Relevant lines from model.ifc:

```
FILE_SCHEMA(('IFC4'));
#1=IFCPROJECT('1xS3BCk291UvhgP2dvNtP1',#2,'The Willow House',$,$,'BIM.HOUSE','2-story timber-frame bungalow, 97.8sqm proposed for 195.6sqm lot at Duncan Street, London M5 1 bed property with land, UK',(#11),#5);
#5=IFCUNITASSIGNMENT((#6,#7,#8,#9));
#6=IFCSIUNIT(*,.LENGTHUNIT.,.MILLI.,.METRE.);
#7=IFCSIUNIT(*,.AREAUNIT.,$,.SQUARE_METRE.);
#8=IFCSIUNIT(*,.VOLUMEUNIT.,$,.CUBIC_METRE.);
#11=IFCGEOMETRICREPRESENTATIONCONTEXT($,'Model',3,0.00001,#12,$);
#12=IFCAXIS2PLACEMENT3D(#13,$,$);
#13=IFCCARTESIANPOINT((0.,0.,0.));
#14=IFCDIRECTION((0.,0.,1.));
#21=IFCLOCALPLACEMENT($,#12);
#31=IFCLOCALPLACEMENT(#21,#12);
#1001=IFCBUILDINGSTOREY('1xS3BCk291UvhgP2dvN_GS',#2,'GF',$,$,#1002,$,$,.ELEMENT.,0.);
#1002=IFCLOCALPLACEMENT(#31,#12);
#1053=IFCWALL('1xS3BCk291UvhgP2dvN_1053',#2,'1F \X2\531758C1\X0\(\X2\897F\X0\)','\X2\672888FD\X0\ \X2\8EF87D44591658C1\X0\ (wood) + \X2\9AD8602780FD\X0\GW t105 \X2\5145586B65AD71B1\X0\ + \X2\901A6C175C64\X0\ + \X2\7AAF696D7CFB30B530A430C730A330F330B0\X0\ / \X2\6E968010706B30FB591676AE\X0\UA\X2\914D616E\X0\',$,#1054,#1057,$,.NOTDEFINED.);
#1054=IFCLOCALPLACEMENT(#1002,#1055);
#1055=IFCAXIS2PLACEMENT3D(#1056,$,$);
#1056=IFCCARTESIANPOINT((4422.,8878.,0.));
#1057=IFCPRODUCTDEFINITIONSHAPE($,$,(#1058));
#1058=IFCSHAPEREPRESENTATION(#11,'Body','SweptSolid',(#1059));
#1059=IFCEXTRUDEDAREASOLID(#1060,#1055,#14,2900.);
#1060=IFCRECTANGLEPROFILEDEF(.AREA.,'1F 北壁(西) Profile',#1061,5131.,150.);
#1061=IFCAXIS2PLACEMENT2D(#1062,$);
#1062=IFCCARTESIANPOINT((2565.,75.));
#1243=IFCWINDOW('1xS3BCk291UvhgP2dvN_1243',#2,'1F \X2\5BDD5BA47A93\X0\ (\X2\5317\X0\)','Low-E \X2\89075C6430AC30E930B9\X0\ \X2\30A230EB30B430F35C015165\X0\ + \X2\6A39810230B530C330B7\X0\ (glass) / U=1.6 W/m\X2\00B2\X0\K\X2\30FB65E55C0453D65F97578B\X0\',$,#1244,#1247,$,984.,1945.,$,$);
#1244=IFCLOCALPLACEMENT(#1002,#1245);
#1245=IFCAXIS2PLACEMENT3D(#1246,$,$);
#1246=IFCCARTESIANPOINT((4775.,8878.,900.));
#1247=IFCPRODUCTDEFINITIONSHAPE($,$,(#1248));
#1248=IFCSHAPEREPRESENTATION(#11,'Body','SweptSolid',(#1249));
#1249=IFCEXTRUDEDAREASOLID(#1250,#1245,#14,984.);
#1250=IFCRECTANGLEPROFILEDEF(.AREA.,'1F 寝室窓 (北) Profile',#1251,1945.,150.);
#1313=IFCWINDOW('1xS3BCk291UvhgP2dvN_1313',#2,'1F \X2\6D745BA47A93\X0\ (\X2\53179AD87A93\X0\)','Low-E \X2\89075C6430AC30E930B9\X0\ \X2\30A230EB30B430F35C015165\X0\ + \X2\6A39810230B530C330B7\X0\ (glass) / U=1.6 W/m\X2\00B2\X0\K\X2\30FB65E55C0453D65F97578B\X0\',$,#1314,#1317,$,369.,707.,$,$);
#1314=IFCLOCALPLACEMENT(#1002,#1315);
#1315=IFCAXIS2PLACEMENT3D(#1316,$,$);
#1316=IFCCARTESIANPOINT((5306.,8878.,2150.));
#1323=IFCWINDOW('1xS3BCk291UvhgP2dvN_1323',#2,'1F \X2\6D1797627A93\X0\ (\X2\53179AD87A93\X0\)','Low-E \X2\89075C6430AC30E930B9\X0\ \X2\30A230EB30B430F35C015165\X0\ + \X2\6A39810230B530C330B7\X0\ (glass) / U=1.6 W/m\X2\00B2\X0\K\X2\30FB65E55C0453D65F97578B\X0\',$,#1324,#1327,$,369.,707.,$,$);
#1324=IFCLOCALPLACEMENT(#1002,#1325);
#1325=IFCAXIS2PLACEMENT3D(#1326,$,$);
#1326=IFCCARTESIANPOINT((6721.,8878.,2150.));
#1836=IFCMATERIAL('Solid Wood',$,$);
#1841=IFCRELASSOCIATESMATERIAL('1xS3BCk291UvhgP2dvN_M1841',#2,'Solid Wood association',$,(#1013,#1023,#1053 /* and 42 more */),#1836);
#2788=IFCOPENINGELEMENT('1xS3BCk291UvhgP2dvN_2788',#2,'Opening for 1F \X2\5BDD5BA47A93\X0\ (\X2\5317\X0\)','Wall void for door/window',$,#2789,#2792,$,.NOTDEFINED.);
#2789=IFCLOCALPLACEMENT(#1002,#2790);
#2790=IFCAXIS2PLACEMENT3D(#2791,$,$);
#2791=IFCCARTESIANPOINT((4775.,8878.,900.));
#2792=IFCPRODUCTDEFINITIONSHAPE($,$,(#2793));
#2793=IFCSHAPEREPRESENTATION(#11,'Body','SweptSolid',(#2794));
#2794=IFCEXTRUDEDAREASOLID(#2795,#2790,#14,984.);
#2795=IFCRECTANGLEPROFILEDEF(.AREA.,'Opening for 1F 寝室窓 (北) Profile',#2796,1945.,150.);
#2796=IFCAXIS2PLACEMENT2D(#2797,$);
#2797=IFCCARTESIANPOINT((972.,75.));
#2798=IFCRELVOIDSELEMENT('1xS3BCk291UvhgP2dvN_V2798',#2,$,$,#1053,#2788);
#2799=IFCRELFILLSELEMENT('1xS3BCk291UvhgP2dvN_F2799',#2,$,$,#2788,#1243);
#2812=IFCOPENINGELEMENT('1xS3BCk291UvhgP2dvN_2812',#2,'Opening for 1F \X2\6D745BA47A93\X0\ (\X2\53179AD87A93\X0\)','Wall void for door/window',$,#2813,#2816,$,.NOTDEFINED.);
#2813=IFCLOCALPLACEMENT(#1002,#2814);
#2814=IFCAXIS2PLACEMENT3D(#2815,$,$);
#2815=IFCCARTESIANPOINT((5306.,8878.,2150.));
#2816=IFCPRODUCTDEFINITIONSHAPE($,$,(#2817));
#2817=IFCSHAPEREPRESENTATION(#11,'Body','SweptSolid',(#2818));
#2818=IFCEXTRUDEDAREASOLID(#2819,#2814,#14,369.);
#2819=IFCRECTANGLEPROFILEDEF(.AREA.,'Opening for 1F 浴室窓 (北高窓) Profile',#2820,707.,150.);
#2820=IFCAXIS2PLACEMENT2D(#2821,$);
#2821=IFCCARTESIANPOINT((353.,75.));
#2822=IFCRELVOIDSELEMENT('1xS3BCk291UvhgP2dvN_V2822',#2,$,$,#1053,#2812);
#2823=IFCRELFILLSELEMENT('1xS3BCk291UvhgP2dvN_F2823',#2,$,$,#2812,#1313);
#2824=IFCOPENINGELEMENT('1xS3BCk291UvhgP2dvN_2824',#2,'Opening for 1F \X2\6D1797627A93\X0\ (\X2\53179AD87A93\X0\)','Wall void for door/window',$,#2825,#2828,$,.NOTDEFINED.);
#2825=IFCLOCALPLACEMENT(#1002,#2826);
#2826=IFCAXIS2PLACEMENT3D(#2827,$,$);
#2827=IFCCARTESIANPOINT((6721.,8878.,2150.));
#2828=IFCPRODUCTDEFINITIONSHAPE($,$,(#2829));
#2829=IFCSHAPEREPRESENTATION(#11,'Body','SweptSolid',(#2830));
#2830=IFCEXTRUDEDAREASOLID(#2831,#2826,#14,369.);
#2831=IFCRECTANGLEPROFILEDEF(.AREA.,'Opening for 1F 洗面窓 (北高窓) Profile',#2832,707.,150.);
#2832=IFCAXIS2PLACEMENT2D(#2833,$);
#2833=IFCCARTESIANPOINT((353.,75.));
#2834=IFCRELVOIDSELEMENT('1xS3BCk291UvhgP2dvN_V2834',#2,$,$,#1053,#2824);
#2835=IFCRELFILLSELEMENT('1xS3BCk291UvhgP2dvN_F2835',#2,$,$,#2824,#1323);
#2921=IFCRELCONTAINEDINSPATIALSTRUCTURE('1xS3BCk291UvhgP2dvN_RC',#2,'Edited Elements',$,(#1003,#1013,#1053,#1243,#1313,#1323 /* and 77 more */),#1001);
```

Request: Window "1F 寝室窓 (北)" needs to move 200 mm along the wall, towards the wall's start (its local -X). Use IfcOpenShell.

```python
import ifcopenshell
import ifcopenshell.api.geometry
import ifcopenshell.util.placement

model = ifcopenshell.open("model.ifc")

window = model.by_guid("1xS3BCk291UvhgP2dvN_1243")
opening = window.FillsVoids[0].RelatingOpeningElement
wall = opening.VoidsElements[0].RelatingBuildingElement

wall_matrix = ifcopenshell.util.placement.get_local_placement(wall.ObjectPlacement)
shift = wall_matrix[:3, 0] * -200.0
before = ifcopenshell.util.placement.get_local_placement(window.ObjectPlacement)[:3, 3].copy()

# The window is not placed relative to its opening, so move both.
for product in (opening, window):
    matrix = ifcopenshell.util.placement.get_local_placement(product.ObjectPlacement)
    matrix[:3, 3] += shift
    ifcopenshell.api.geometry.edit_object_placement(model, product=product, matrix=matrix, is_si=False)

after = ifcopenshell.util.placement.get_local_placement(window.ObjectPlacement)[:3, 3]
print("window moved by", (after - before).round(3) + 0.0)

model.write("model_v2.ifc")
```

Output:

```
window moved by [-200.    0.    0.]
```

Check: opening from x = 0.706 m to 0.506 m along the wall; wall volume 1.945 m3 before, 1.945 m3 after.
